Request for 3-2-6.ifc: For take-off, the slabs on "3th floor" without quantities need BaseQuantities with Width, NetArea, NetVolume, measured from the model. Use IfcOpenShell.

First a look at what the model holds.

```python
import ifcopenshell
import ifcopenshell.util.element
import ifcopenshell.util.unit

model = ifcopenshell.open("3-2-6.ifc")
print(model.schema)
for unit_type in ("LENGTHUNIT", "AREAUNIT", "VOLUMEUNIT"):
    print(unit_type, ifcopenshell.util.unit.calculate_unit_scale(model, unit_type))
storey = next(s for s in model.by_type("IfcBuildingStorey") if s.Name == "3th floor")
slabs = [e for e in ifcopenshell.util.element.get_decomposition(storey) if e.is_a("IfcSlab")]
for e in sorted(slabs, key=lambda e: e.id()):
    print(e.id(), e.is_a(), e.Name, list(ifcopenshell.util.element.get_psets(e, qtos_only=True)), sep=" | ")
```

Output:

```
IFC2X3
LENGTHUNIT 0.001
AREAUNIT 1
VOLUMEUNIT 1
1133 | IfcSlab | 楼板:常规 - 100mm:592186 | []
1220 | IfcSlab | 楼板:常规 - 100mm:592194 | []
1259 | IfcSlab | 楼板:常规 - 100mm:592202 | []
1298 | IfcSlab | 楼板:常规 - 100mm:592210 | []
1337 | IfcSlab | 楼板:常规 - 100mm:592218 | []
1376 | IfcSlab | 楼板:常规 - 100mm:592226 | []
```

```python
import ifcopenshell
import ifcopenshell.api.pset
import ifcopenshell.geom
import ifcopenshell.util.element
import ifcopenshell.util.shape
import ifcopenshell.util.unit

model = ifcopenshell.open("3-2-6.ifc")
unit_scale = ifcopenshell.util.unit.calculate_unit_scale(model)
area_scale = ifcopenshell.util.unit.calculate_unit_scale(model, "AREAUNIT")
volume_scale = ifcopenshell.util.unit.calculate_unit_scale(model, "VOLUMEUNIT")
settings = ifcopenshell.geom.settings()

storey = next(s for s in model.by_type("IfcBuildingStorey") if s.Name == "3th floor")
slabs = [e for e in ifcopenshell.util.element.get_decomposition(storey) if e.is_a("IfcSlab")]

for e in sorted(slabs, key=lambda e: e.id()):
    if ifcopenshell.util.element.get_psets(e, qtos_only=True, should_inherit=False):
        continue
    # Geometry comes back in metres, in the element's own axes.
    shape = ifcopenshell.geom.create_shape(settings, e)
    values = {
        "Width": ifcopenshell.util.shape.get_z(shape.geometry) / unit_scale,
        "NetArea": ifcopenshell.util.shape.get_footprint_area(shape.geometry) / area_scale,
        "NetVolume": ifcopenshell.util.shape.get_volume(shape.geometry) / volume_scale,
    }
    qto = ifcopenshell.api.pset.add_qto(model, product=e, name="BaseQuantities")
    ifcopenshell.api.pset.edit_qto(model, qto=qto, properties=values)
    print(e.id(), {k: round(v, 3) for k, v in values.items()})

model.write("3-2-6_edited.ifc")
```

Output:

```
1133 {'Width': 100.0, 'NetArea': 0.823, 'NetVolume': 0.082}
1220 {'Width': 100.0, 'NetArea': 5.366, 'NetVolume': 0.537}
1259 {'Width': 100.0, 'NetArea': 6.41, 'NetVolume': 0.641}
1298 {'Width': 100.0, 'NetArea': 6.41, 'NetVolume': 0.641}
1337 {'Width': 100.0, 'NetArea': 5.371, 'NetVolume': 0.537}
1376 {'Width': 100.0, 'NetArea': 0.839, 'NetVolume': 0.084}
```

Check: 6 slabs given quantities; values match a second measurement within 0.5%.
